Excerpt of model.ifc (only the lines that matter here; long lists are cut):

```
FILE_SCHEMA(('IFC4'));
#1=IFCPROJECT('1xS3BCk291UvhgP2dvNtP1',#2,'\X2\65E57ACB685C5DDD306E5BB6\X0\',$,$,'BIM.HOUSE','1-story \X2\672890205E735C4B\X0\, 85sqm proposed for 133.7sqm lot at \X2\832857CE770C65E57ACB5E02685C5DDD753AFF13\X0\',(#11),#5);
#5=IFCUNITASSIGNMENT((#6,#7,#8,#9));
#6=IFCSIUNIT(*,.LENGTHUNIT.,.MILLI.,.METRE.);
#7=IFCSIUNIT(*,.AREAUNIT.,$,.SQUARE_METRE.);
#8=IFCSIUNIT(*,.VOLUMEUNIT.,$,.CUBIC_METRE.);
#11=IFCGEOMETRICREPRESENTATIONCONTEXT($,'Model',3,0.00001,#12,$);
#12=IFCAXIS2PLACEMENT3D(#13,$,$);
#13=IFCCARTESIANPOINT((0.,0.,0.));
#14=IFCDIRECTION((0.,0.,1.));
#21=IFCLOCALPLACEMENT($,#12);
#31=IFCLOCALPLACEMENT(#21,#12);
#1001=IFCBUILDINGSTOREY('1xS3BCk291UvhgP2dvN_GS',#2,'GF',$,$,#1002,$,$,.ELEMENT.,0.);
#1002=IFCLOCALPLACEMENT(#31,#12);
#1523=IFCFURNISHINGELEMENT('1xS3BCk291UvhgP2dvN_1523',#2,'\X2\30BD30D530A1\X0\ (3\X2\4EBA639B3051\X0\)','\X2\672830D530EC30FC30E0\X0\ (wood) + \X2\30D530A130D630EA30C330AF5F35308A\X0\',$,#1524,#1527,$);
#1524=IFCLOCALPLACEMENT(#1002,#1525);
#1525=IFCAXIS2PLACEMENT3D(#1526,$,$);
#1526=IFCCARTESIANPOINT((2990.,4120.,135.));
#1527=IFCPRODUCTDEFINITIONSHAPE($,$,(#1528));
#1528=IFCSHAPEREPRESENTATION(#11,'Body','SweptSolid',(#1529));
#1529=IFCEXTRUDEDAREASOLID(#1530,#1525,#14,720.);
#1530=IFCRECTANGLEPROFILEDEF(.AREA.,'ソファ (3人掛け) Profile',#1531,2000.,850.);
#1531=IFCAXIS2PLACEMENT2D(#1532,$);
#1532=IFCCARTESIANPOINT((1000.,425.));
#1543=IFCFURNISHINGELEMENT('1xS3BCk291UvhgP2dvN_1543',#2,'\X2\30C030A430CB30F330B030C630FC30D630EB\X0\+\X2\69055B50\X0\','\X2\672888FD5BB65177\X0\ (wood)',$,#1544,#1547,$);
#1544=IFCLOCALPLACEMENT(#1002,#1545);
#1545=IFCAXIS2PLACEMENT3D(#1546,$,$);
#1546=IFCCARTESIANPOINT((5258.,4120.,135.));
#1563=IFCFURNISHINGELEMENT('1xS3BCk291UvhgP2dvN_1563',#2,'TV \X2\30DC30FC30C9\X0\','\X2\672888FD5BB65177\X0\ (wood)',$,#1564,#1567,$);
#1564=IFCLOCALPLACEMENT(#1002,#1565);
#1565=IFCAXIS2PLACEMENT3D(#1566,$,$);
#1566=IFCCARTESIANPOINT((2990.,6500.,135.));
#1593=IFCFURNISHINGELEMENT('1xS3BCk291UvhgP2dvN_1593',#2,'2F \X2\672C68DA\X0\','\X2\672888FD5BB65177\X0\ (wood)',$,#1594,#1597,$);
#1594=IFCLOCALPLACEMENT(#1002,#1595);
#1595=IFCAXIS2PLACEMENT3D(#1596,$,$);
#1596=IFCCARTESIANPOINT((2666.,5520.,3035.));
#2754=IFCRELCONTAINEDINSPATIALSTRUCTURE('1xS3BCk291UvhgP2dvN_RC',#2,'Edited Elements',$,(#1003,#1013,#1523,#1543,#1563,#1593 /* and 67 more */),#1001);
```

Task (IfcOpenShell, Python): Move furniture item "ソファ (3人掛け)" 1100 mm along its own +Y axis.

```python
import ifcopenshell
import ifcopenshell.api.geometry
import ifcopenshell.util.placement

model = ifcopenshell.open("model.ifc")

item = model.by_guid("1xS3BCk291UvhgP2dvN_1523")
matrix = ifcopenshell.util.placement.get_local_placement(item.ObjectPlacement)
matrix[:3, 3] += matrix[:3, 1] * 1100.0
ifcopenshell.api.geometry.edit_object_placement(model, product=item, matrix=matrix, is_si=False)

print(ifcopenshell.util.placement.get_local_placement(item.ObjectPlacement).round(3) + 0.0)

model.write("model_edited.ifc")
```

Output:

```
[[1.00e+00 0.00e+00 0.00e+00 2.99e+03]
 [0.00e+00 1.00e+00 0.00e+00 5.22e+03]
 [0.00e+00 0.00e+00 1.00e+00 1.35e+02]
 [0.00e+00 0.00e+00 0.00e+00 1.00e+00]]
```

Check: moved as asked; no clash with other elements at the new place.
